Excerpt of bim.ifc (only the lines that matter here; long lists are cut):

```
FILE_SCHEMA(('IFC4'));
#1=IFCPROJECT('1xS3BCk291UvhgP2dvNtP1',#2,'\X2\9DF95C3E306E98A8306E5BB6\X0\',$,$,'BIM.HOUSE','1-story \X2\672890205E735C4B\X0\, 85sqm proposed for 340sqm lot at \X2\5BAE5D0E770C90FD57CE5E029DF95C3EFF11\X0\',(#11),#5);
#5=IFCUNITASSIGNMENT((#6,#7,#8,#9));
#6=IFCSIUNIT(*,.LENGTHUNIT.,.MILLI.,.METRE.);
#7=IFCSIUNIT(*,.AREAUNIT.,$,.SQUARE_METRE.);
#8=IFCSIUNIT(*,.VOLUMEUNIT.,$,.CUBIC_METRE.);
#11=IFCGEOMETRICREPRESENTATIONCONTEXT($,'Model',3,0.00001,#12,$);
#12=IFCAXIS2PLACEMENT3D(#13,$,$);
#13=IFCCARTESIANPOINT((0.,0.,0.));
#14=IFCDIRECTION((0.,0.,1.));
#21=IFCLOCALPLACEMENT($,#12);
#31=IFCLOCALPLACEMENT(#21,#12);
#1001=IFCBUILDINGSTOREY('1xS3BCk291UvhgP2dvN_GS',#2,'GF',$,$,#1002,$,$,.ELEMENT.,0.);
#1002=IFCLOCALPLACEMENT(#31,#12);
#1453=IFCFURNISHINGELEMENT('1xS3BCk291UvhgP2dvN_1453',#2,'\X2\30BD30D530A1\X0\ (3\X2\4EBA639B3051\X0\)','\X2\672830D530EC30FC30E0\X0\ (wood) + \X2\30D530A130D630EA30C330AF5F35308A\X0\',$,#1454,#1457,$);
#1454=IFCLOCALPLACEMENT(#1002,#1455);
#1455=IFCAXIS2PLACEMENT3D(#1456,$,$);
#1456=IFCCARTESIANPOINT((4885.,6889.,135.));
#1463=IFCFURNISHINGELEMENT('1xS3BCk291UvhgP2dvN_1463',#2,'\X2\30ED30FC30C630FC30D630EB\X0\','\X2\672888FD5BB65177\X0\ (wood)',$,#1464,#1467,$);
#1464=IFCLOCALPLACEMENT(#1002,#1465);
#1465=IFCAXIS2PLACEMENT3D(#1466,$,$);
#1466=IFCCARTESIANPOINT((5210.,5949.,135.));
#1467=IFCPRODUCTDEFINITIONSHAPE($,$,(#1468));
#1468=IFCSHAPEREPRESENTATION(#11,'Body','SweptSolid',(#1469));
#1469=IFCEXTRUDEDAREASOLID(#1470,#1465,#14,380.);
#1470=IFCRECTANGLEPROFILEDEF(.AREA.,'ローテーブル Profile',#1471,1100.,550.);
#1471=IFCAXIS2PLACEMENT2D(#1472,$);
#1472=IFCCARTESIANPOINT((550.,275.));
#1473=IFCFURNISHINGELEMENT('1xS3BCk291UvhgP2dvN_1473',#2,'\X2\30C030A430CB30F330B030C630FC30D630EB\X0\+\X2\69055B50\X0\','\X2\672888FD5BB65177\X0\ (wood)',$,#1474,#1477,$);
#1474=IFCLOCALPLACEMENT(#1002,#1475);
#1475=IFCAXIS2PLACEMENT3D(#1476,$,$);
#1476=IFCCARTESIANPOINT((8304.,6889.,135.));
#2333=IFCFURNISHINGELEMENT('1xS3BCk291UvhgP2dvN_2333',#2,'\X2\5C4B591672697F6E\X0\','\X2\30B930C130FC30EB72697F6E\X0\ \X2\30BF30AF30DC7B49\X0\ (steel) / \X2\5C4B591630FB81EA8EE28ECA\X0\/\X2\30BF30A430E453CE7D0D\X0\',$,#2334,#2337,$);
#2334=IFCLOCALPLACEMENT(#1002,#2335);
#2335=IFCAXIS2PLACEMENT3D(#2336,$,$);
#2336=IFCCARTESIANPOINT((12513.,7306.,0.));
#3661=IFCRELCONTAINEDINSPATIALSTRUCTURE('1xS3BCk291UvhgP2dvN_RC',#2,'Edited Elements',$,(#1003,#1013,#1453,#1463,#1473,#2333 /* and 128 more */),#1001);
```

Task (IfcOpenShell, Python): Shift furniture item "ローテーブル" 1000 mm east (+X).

```python
import ifcopenshell
import ifcopenshell.api.geometry
import ifcopenshell.util.placement

model = ifcopenshell.open("bim.ifc")

item = model.by_guid("1xS3BCk291UvhgP2dvN_1463")
matrix = ifcopenshell.util.placement.get_local_placement(item.ObjectPlacement)
matrix[0, 3] += 1000.0
ifcopenshell.api.geometry.edit_object_placement(model, product=item, matrix=matrix, is_si=False)

print(ifcopenshell.util.placement.get_local_placement(item.ObjectPlacement).round(3) + 0.0)

model.write("bim_rev.ifc")
```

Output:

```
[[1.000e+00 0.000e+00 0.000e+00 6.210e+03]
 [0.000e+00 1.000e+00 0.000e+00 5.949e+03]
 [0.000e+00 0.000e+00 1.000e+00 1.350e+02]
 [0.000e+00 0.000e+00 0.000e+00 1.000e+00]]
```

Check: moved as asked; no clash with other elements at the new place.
